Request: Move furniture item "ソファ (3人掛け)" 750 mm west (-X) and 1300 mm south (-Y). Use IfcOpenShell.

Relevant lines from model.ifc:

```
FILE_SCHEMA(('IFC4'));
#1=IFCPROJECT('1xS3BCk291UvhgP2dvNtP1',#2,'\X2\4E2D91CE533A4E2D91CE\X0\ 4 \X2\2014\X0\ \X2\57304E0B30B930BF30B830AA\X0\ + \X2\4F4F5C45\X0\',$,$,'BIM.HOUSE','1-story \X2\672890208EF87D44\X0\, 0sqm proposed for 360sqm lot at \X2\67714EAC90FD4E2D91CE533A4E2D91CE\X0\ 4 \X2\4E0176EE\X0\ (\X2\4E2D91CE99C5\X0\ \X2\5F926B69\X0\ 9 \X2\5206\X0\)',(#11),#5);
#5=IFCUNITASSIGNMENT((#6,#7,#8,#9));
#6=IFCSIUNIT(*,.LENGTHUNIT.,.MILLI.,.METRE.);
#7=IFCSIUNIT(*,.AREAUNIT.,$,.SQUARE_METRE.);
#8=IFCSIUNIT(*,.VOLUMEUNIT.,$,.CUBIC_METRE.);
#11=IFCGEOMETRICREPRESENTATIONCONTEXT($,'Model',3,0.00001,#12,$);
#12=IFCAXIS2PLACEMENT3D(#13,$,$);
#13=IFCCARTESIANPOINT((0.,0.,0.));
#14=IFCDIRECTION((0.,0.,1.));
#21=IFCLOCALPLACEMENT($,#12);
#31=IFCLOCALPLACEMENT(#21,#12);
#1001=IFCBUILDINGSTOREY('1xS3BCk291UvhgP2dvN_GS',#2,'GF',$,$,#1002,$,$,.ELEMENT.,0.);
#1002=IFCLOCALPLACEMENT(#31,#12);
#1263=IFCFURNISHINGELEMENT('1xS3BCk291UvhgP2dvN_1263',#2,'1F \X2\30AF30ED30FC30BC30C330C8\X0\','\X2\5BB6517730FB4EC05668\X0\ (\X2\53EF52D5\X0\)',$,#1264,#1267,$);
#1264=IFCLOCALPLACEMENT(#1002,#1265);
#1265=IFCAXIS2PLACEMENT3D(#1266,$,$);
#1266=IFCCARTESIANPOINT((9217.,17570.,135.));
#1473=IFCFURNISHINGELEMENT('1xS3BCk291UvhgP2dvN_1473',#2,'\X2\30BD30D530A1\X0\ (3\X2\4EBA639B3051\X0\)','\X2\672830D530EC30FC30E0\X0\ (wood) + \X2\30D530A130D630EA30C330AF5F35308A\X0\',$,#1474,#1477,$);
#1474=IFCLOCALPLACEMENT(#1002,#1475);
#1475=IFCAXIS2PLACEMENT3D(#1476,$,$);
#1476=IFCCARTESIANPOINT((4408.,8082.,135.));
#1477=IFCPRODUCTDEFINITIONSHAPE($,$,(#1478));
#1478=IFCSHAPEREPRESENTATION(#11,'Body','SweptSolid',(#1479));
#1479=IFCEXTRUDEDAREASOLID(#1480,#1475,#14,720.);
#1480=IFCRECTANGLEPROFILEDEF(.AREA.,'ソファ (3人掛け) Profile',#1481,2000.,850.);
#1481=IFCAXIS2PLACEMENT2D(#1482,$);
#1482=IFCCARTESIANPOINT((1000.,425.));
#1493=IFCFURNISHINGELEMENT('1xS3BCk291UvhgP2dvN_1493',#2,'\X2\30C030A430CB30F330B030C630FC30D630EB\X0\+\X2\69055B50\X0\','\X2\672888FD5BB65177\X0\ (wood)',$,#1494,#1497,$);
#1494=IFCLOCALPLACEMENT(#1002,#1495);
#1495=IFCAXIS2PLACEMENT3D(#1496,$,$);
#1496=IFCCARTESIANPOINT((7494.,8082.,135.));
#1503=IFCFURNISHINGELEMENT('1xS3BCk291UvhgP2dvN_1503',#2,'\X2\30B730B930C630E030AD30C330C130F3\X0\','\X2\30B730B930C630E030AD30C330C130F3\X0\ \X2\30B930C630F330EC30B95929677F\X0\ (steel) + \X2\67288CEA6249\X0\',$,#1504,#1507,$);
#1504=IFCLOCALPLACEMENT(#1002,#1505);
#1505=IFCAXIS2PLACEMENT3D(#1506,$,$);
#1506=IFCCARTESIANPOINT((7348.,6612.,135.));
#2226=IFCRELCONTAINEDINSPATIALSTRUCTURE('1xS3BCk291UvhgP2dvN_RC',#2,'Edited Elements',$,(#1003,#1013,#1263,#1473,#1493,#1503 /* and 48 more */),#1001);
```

```python
import ifcopenshell
import ifcopenshell.api.geometry
import ifcopenshell.util.placement
import ifcopenshell.util.unit

model = ifcopenshell.open("model.ifc")
unit_scale = ifcopenshell.util.unit.calculate_unit_scale(model)

item = model.by_id(1473)
matrix = ifcopenshell.util.placement.get_local_placement(item.ObjectPlacement)
matrix[0, 3] -= 0.75 / unit_scale
matrix[1, 3] -= 1.3 / unit_scale
ifcopenshell.api.geometry.edit_object_placement(model, product=item, matrix=matrix, is_si=False)

print(ifcopenshell.util.placement.get_local_placement(item.ObjectPlacement).round(3) + 0.0)

model.write("model-out.ifc")
```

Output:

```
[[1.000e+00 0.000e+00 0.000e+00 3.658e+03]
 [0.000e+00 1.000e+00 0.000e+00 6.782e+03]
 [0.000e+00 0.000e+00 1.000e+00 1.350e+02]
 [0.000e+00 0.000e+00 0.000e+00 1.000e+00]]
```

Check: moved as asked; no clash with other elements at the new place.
